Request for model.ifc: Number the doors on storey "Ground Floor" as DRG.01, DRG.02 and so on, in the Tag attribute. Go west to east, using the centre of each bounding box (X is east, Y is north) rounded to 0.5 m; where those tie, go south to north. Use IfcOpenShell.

First a look at what the model holds.

```python
import ifcopenshell
import ifcopenshell.util.element
import ifcopenshell.util.placement

model = ifcopenshell.open("model.ifc")
print(model.schema)
storey = next(s for s in model.by_type("IfcBuildingStorey") if s.Name == "Ground Floor")
doors = [e for e in ifcopenshell.util.element.get_decomposition(storey) if e.is_a("IfcDoor")]
for e in sorted(doors, key=lambda e: e.id()):
    origin = ifcopenshell.util.placement.get_local_placement(e.ObjectPlacement)[:3, 3]
    print(e.id(), e.Tag, e.Name, origin.round(2) + 0.0, sep=" | ")
```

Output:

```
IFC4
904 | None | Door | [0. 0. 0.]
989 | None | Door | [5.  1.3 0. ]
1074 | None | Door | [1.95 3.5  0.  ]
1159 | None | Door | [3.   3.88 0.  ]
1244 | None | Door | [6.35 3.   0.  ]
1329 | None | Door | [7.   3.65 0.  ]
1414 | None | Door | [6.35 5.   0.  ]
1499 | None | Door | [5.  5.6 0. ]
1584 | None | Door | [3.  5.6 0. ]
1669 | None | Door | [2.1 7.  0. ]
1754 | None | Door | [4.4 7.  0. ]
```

```python
import ifcopenshell
import ifcopenshell.geom
import ifcopenshell.util.element
import ifcopenshell.util.shape

model = ifcopenshell.open("model.ifc")
settings = ifcopenshell.geom.settings()
settings.set("use-world-coords", True)


def centre(element):
    shape = ifcopenshell.geom.create_shape(settings, element)
    return ifcopenshell.util.shape.get_bbox_centroid(shape.geometry)


storey = next(s for s in model.by_type("IfcBuildingStorey") if s.Name == "Ground Floor")
doors = [e for e in ifcopenshell.util.element.get_decomposition(storey) if e.is_a("IfcDoor")]

# Insertion points can sit at a corner or the storey origin, so sort by the geometry (in metres).
centres = {e: centre(e) for e in doors}
doors.sort(key=lambda e: (round(centres[e][0] / 0.5), centres[e][1]))

for i, e in enumerate(doors, start=1):
    number = f"DRG.{i:02d}"
    e.Tag = number
    print(e.id(), number)

model.write("model_edited.ifc")
```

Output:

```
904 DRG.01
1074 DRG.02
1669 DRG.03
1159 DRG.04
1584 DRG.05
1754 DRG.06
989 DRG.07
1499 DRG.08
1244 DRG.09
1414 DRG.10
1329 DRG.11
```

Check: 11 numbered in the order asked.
